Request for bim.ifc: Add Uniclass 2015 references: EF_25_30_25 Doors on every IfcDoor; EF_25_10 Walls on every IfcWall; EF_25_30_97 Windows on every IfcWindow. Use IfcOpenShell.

First a look at what the model holds.

```python
import ifcopenshell

model = ifcopenshell.open("bim.ifc")
print(model.schema)
print("classifications:", [c.Name for c in model.by_type("IfcClassification")])
for ifc_class in ("IfcDoor", "IfcRoof", "IfcStair", "IfcWall", "IfcWindow"):
    print(ifc_class, len(model.by_type(ifc_class)))
```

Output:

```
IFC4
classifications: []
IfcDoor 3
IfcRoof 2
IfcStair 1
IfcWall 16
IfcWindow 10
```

```python
import ifcopenshell
import ifcopenshell.api.classification

model = ifcopenshell.open("bim.ifc")

system = ifcopenshell.api.classification.add_classification(model, classification="Uniclass 2015")

codes = {
    "IfcDoor": ("EF_25_30_25", "Doors"),
    "IfcWall": ("EF_25_10", "Walls"),
    "IfcWindow": ("EF_25_30_97", "Windows"),
}
for ifc_class, (code, name) in codes.items():
    products = model.by_type(ifc_class)
    ifcopenshell.api.classification.add_reference(
        model, products=products, classification=system, identification=code, name=name
    )
    print(code, len(products))

model.write("bim_rev.ifc")
```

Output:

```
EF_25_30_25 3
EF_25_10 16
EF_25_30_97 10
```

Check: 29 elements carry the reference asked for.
